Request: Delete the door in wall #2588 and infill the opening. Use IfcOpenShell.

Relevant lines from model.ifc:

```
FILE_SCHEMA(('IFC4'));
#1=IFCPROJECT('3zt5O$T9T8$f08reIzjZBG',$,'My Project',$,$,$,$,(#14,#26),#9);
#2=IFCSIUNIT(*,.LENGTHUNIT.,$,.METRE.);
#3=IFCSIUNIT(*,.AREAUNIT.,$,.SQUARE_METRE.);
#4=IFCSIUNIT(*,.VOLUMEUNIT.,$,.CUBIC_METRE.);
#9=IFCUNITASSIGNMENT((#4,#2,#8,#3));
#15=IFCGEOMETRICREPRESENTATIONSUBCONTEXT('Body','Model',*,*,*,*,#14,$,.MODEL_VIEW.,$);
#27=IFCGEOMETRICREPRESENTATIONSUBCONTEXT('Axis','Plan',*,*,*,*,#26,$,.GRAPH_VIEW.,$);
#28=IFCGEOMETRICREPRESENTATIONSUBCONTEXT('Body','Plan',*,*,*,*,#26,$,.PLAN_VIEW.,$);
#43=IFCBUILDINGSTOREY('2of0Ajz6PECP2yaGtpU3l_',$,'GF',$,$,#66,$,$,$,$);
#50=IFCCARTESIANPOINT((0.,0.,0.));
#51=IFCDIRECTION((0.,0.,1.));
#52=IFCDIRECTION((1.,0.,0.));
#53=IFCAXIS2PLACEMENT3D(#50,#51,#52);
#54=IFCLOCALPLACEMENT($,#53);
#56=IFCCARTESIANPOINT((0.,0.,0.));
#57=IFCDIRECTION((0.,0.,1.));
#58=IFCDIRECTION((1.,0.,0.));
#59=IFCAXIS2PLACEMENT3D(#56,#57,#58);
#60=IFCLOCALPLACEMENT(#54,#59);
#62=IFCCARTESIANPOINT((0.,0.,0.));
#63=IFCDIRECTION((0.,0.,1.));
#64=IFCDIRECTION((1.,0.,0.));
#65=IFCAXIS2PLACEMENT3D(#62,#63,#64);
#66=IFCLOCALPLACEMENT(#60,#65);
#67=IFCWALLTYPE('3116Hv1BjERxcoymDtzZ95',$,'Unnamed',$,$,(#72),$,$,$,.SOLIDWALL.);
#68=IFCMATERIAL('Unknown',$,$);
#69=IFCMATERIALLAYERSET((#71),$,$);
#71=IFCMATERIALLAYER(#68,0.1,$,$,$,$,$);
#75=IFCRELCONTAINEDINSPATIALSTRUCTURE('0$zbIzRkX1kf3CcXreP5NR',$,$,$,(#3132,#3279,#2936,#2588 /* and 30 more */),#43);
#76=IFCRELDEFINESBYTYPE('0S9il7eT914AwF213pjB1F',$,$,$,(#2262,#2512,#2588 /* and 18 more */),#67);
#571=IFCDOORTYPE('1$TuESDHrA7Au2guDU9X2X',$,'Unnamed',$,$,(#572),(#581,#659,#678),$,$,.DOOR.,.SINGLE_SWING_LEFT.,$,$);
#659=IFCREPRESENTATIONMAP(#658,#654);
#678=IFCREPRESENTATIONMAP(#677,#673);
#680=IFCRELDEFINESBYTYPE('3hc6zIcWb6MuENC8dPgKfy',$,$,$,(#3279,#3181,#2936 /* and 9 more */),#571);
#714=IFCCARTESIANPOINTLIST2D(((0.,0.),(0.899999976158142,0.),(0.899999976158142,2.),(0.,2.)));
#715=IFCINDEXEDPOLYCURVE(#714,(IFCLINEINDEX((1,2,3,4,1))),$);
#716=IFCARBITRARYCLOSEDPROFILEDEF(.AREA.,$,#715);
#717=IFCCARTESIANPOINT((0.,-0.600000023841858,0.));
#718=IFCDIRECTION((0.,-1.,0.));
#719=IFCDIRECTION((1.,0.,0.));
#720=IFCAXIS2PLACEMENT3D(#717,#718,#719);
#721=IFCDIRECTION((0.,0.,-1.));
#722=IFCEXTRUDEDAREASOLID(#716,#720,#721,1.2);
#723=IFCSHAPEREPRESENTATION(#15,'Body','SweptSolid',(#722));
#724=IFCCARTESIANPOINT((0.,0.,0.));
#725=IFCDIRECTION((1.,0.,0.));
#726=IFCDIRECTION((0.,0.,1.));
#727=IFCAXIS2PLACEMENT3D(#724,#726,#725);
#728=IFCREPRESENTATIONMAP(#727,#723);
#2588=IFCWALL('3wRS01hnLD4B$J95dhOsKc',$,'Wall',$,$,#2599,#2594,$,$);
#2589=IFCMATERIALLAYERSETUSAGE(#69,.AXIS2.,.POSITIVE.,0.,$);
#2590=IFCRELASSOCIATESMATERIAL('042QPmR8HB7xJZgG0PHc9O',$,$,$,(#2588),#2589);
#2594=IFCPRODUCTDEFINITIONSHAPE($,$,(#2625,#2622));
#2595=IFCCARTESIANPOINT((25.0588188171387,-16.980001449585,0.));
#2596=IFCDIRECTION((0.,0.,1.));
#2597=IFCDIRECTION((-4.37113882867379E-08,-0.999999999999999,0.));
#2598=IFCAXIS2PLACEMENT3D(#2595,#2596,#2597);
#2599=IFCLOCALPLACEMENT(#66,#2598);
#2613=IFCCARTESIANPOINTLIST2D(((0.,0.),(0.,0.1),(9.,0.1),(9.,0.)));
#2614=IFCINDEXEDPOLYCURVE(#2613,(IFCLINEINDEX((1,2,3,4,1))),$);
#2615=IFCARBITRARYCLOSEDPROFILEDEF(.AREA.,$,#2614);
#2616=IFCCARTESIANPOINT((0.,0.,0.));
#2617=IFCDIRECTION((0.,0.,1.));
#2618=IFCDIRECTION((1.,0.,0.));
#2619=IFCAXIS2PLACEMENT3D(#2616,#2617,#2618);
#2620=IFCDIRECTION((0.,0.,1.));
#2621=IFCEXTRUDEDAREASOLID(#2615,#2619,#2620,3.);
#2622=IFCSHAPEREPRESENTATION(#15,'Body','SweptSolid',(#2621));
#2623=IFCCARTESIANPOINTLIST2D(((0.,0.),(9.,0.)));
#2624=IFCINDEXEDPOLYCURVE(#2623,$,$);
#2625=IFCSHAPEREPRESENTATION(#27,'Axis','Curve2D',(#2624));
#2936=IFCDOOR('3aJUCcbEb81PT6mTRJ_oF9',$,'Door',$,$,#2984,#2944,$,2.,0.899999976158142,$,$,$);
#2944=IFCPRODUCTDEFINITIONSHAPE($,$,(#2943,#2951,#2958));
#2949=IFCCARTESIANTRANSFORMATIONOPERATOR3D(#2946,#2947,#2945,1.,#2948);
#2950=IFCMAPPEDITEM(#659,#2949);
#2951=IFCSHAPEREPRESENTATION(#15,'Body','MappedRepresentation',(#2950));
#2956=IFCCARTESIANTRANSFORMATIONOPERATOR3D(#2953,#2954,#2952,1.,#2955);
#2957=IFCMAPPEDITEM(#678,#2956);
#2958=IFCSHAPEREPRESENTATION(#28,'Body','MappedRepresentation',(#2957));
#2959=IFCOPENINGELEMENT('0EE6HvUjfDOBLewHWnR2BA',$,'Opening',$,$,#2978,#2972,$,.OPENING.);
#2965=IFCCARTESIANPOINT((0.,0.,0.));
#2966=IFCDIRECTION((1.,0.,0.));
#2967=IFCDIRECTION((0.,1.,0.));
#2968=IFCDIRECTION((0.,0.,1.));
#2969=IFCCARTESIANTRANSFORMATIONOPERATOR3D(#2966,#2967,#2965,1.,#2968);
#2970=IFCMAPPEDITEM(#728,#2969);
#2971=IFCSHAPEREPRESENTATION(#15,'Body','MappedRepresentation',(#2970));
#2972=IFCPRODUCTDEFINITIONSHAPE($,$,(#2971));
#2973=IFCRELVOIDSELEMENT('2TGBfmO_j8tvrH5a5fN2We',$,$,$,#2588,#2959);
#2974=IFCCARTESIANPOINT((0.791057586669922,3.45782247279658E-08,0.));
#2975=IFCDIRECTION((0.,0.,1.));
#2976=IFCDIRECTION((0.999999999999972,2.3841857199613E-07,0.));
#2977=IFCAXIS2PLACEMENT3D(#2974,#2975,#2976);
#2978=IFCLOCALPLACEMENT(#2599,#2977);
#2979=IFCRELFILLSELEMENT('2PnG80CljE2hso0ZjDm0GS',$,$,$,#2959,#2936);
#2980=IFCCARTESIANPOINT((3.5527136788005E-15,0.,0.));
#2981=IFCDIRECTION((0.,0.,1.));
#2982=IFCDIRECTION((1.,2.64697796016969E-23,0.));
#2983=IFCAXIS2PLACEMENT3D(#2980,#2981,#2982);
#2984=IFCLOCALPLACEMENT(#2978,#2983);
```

```python
import ifcopenshell
import ifcopenshell.api.feature
import ifcopenshell.api.root
import ifcopenshell.geom
import ifcopenshell.util.shape

model = ifcopenshell.open("model.ifc")
settings = ifcopenshell.geom.settings()


def volume(element):
    """Net volume in cubic metres, openings subtracted."""
    shape = ifcopenshell.geom.create_shape(settings, element)
    return ifcopenshell.util.shape.get_volume(shape.geometry)


door = model.by_guid("3aJUCcbEb81PT6mTRJ_oF9")
opening = door.FillsVoids[0].RelatingOpeningElement
wall = opening.VoidsElements[0].RelatingBuildingElement
before = volume(wall)

ifcopenshell.api.root.remove_product(model, product=door)
ifcopenshell.api.feature.remove_feature(model, feature=opening)

after = volume(wall)

print(f"wall volume {before:.3f} -> {after:.3f} m3")

model.write("model_rev.ifc")
```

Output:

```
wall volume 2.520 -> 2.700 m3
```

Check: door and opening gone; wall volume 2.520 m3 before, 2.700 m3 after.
